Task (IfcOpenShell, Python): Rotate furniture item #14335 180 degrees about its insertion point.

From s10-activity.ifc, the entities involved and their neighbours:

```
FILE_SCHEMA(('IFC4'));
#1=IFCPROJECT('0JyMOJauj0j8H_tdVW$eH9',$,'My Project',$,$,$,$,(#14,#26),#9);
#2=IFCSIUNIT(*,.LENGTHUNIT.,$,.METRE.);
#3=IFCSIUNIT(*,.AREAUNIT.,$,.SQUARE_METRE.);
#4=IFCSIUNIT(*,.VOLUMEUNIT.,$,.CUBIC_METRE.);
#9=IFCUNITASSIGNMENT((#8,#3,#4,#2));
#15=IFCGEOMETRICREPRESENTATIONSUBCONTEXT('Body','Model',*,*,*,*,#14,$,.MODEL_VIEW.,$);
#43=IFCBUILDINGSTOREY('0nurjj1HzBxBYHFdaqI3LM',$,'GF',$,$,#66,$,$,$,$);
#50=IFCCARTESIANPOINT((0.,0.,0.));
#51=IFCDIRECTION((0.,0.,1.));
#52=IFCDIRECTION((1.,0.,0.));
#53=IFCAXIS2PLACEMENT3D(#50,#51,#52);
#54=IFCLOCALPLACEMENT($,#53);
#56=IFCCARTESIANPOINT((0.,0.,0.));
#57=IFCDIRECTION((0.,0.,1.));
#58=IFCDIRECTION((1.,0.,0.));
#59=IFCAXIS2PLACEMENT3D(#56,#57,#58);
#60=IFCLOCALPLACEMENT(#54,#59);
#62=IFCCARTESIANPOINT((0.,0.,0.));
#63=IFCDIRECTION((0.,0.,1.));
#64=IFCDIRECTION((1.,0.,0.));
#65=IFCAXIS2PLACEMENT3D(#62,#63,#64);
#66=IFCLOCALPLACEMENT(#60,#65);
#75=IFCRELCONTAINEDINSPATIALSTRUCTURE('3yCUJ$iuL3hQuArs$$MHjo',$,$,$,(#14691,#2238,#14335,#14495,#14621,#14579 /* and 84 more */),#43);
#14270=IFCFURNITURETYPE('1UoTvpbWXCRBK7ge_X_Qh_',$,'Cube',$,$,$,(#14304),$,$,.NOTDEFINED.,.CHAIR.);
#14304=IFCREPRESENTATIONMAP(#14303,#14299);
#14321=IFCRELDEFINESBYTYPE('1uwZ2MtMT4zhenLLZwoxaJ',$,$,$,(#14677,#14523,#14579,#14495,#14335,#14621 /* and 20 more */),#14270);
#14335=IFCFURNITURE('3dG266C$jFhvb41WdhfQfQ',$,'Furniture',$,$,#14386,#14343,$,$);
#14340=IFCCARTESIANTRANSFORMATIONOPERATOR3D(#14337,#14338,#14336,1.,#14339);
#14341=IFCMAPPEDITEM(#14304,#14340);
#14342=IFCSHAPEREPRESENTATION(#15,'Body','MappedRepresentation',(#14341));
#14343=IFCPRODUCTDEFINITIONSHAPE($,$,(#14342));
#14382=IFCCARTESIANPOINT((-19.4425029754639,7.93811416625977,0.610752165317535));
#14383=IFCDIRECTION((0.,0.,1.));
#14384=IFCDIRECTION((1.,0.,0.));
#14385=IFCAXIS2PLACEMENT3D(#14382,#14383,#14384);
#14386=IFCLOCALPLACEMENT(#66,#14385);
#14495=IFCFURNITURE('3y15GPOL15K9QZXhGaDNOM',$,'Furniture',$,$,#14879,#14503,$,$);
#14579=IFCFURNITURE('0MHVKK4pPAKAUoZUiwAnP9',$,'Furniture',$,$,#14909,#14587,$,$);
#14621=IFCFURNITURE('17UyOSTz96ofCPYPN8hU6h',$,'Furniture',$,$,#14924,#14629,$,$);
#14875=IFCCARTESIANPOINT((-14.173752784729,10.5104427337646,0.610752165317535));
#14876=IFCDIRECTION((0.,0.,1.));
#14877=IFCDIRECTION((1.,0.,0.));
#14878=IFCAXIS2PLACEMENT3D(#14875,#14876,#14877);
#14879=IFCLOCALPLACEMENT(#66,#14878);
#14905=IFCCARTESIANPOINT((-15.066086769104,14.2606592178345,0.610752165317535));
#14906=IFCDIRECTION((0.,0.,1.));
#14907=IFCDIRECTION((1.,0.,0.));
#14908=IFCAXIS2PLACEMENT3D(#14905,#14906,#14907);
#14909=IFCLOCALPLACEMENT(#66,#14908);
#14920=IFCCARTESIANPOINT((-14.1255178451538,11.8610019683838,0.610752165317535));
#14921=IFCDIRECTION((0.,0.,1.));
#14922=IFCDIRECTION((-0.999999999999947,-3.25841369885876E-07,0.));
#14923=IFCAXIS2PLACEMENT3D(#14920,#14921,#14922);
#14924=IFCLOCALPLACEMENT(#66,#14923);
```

```python
import ifcopenshell
import ifcopenshell.api.geometry
import ifcopenshell.util.placement

model = ifcopenshell.open("s10-activity.ifc")

item = model.by_guid("3dG266C$jFhvb41WdhfQfQ")
matrix = ifcopenshell.util.placement.get_local_placement(item.ObjectPlacement)
matrix = matrix @ ifcopenshell.util.placement.rotation(180, "Z")
ifcopenshell.api.geometry.edit_object_placement(model, product=item, matrix=matrix, is_si=False)

print(ifcopenshell.util.placement.get_local_placement(item.ObjectPlacement).round(3) + 0.0)

model.write("s10-activity_edited.ifc")
```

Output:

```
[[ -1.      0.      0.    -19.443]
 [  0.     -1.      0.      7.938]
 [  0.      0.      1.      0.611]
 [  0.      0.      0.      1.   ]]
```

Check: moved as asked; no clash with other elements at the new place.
